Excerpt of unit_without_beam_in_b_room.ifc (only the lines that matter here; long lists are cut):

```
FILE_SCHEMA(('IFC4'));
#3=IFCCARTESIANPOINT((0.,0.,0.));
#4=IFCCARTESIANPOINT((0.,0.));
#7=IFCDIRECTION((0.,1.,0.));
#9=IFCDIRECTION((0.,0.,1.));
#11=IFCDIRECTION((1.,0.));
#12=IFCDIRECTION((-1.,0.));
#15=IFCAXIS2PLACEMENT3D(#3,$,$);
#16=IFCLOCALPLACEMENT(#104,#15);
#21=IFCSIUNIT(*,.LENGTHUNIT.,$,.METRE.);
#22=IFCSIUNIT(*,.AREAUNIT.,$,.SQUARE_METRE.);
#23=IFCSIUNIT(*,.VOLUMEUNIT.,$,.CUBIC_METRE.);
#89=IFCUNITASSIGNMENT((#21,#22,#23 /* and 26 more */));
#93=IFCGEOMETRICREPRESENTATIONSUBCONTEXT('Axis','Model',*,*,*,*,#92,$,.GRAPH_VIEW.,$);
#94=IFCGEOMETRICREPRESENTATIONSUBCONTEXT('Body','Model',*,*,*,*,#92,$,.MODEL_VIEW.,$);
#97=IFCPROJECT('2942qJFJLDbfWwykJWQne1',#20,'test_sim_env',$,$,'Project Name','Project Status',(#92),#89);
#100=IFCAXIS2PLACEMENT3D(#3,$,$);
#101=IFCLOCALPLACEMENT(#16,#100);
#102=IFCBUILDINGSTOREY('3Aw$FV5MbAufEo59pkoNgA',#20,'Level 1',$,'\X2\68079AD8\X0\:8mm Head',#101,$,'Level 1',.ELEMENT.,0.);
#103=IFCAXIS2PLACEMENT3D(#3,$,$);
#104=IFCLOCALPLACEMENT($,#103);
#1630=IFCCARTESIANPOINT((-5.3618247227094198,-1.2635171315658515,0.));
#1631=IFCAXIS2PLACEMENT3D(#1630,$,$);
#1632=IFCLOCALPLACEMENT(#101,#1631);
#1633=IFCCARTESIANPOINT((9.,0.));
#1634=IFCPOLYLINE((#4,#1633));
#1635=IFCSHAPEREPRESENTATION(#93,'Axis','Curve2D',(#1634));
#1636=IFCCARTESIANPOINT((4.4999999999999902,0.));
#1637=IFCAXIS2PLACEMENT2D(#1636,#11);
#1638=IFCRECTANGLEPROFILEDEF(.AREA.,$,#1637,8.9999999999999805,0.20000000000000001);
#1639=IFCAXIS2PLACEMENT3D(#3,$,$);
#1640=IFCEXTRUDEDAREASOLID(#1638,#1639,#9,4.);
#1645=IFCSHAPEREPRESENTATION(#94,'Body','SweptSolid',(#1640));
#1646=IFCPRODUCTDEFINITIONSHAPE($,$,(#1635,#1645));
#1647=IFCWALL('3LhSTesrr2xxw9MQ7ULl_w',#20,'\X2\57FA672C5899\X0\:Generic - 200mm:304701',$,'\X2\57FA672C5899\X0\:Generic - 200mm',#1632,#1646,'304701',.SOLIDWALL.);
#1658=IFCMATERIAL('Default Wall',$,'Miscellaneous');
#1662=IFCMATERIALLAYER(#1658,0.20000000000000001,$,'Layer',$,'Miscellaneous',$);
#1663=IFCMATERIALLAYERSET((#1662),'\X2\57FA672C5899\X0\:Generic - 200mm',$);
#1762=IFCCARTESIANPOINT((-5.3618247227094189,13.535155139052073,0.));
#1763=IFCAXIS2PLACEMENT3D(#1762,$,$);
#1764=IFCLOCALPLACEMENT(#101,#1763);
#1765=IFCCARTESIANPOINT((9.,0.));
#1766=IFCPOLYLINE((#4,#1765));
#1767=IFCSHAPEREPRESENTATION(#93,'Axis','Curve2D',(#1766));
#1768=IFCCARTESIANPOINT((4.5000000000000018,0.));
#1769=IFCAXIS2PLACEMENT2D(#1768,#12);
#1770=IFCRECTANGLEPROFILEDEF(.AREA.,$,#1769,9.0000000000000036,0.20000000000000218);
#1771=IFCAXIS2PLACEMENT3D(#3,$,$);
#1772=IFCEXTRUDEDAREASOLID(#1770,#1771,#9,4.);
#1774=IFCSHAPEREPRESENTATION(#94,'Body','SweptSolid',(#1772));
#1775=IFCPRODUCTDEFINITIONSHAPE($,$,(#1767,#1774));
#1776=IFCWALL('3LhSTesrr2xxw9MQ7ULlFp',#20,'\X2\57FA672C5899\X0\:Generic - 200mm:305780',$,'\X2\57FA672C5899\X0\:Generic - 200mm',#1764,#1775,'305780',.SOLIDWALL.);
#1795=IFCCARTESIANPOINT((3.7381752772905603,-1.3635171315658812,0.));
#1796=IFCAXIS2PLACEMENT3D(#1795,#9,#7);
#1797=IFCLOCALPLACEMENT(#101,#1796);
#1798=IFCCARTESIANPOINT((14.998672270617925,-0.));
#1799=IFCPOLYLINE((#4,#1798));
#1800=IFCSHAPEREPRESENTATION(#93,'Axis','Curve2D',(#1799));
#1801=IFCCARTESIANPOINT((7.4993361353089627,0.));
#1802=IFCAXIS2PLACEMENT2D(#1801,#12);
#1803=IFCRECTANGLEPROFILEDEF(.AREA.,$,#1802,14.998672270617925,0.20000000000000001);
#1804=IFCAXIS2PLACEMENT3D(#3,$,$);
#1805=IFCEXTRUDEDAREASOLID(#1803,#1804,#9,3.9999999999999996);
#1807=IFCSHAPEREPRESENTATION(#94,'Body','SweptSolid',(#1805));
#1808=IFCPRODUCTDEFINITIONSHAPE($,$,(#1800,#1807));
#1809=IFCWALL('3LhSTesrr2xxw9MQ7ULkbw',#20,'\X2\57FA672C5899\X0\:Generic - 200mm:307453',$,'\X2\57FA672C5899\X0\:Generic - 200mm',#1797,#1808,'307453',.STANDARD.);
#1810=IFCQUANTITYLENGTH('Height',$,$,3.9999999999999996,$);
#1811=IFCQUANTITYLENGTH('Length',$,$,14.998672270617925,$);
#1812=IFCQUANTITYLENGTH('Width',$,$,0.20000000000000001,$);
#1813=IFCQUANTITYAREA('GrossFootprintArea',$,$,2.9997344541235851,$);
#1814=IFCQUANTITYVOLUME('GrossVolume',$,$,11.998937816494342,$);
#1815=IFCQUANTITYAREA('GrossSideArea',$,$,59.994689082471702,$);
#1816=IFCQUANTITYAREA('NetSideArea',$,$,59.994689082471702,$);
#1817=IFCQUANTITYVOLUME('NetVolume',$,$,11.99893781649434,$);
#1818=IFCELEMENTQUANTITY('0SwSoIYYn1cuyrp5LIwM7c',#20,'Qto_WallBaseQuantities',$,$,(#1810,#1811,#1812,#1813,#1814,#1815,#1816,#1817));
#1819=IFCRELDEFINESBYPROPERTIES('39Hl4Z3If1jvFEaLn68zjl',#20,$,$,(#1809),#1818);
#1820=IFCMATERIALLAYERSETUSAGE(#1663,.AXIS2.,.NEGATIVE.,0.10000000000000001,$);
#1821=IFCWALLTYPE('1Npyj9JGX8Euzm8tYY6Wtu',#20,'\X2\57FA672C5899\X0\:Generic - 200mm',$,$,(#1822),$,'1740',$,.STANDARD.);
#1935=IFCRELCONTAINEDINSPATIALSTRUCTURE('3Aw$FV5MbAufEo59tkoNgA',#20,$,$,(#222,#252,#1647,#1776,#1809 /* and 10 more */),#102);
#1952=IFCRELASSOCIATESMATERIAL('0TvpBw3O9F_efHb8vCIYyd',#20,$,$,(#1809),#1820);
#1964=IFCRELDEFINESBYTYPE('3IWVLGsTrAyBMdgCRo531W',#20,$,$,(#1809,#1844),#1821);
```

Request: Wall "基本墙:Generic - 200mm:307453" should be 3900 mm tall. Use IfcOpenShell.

```python
import ifcopenshell
import ifcopenshell.api.pset
import ifcopenshell.geom
import ifcopenshell.util.element
import ifcopenshell.util.representation
import ifcopenshell.util.shape
import ifcopenshell.util.unit

model = ifcopenshell.open("unit_without_beam_in_b_room.ifc")
unit_scale = ifcopenshell.util.unit.calculate_unit_scale(model)
area_scale = ifcopenshell.util.unit.calculate_unit_scale(model, "AREAUNIT")
volume_scale = ifcopenshell.util.unit.calculate_unit_scale(model, "VOLUMEUNIT")
settings = ifcopenshell.geom.settings()


def volume(element):
    """Net volume in cubic metres, openings subtracted."""
    shape = ifcopenshell.geom.create_shape(settings, element)
    return ifcopenshell.util.shape.get_volume(shape.geometry)


wall = model.by_guid("3LhSTesrr2xxw9MQ7ULkbw")
before = volume(wall)

body = ifcopenshell.util.representation.get_representation(wall, "Model", "Body")
solid = body.Items[0]
old_height = solid.Depth
solid.Depth = 3.9 / unit_scale
after = volume(wall)
thickness = 0.2  # wall thickness in metres

# Update the stored height, areas and volumes.
qto = model.by_id(ifcopenshell.util.element.get_pset(wall, "Qto_WallBaseQuantities", should_inherit=False)["id"])
ifcopenshell.api.pset.edit_qto(model, qto=qto, properties={
    "Height": solid.Depth,
    "GrossVolume": ifcopenshell.util.element.get_pset(wall, "Qto_WallBaseQuantities", "GrossVolume") * solid.Depth / old_height,
    "GrossSideArea": ifcopenshell.util.element.get_pset(wall, "Qto_WallBaseQuantities", "GrossSideArea") * solid.Depth / old_height,
    "NetSideArea": after / thickness / area_scale,
    "NetVolume": after / volume_scale,
})

print(f"height {old_height:g} -> {solid.Depth:g}, volume {before:.3f} -> {after:.3f} m3")

model.write("unit_without_beam_in_b_room_edited.ifc")
```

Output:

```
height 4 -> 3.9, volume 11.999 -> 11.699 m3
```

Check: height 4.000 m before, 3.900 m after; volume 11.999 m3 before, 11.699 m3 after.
